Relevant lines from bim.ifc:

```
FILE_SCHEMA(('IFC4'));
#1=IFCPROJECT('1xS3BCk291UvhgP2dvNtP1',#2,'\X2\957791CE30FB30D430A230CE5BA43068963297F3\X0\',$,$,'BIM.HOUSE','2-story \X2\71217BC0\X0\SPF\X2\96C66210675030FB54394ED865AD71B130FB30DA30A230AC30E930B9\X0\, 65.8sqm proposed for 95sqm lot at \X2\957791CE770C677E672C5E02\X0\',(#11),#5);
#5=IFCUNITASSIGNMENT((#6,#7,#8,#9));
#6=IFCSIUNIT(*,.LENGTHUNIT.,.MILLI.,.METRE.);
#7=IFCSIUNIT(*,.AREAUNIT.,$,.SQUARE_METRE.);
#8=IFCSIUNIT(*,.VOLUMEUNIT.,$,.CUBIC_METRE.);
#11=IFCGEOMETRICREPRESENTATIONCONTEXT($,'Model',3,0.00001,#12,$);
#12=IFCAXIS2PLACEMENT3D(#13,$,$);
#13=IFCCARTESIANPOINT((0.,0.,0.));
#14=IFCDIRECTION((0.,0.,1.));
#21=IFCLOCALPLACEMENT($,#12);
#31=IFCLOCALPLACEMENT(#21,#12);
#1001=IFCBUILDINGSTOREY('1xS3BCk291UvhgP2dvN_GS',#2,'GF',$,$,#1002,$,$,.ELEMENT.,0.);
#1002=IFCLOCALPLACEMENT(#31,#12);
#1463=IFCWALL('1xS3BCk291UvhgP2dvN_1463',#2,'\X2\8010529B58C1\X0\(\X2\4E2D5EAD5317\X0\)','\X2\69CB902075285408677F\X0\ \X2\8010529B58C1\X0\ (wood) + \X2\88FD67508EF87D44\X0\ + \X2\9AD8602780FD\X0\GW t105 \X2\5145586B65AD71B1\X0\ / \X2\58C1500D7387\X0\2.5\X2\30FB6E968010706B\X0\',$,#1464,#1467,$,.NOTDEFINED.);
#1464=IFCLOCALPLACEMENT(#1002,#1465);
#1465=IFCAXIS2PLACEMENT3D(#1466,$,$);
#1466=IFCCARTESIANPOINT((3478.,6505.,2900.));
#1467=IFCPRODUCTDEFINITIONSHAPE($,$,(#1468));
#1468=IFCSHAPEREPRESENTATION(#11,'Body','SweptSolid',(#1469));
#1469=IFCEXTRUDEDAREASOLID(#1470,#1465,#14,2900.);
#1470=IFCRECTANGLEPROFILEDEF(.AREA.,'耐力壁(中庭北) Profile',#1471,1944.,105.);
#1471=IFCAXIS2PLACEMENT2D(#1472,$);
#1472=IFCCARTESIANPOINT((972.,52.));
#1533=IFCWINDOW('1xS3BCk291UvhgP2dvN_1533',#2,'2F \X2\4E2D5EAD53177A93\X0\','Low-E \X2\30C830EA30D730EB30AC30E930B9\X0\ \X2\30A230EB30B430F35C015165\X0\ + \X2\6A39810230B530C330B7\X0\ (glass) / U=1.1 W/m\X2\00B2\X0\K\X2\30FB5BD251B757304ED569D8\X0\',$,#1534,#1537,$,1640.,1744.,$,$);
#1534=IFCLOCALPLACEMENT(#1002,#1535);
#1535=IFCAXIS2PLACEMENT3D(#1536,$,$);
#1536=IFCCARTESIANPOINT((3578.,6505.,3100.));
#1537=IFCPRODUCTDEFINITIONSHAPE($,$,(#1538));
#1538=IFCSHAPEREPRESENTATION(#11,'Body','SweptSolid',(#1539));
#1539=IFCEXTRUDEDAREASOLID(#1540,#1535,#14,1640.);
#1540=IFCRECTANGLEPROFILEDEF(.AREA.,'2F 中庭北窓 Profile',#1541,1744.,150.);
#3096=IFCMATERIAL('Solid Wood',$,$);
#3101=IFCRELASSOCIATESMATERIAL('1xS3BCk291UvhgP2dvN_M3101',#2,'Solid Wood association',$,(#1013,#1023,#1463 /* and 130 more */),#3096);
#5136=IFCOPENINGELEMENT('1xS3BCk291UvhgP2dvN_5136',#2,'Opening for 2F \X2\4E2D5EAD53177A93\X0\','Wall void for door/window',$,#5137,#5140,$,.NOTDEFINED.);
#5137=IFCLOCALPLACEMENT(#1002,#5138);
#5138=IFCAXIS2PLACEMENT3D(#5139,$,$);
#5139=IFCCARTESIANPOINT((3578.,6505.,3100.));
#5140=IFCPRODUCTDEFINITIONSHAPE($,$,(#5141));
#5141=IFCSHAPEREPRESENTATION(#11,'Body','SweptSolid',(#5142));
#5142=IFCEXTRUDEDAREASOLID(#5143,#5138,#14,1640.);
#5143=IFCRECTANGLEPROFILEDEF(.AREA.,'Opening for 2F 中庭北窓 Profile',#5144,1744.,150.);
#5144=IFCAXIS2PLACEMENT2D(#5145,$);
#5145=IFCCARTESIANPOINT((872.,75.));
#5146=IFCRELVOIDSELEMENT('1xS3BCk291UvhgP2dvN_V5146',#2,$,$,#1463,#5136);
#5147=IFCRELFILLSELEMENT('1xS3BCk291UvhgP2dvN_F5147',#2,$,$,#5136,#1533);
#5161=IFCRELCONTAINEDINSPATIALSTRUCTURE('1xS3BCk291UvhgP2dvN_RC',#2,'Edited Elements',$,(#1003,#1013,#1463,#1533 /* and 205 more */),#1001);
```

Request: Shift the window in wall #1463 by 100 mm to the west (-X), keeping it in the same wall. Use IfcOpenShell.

```python
import ifcopenshell
import ifcopenshell.api.geometry
import ifcopenshell.util.placement
import ifcopenshell.util.unit

model = ifcopenshell.open("bim.ifc")
unit_scale = ifcopenshell.util.unit.calculate_unit_scale(model)

window = model.by_id(1533)
opening = window.FillsVoids[0].RelatingOpeningElement
wall = opening.VoidsElements[0].RelatingBuildingElement

wall_matrix = ifcopenshell.util.placement.get_local_placement(wall.ObjectPlacement)
shift = wall_matrix[:3, 0] * -0.1 / unit_scale
before = ifcopenshell.util.placement.get_local_placement(window.ObjectPlacement)[:3, 3].copy()

# The window is not placed relative to its opening, so move both.
for product in (opening, window):
    matrix = ifcopenshell.util.placement.get_local_placement(product.ObjectPlacement)
    matrix[:3, 3] += shift
    ifcopenshell.api.geometry.edit_object_placement(model, product=product, matrix=matrix, is_si=False)

after = ifcopenshell.util.placement.get_local_placement(window.ObjectPlacement)[:3, 3]
print("window moved by", (after - before).round(3) + 0.0)

model.write("bim-out.ifc")
```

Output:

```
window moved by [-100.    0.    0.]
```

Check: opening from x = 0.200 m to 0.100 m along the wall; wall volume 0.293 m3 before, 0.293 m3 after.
